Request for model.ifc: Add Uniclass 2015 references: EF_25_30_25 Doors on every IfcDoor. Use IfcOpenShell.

First a look at what the model holds.

```python
import ifcopenshell

model = ifcopenshell.open("model.ifc")
print(model.schema)
print("classifications:", [c.Name for c in model.by_type("IfcClassification")])
for ifc_class in ("IfcDoor", "IfcRoof", "IfcStair", "IfcWall", "IfcWindow"):
    print(ifc_class, len(model.by_type(ifc_class)))
```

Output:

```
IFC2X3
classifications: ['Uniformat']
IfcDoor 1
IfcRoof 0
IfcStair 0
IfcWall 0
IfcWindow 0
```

```python
import ifcopenshell
import ifcopenshell.api.classification

model = ifcopenshell.open("model.ifc")

# IFC2X3 requires Source and Edition and has no link from the project to the system.
system = model.create_entity("IfcClassification", Source="NBS", Edition="2015", Name="Uniclass 2015")

codes = {
    "IfcDoor": ("EF_25_30_25", "Doors"),
}
for ifc_class, (code, name) in codes.items():
    products = model.by_type(ifc_class)
    ifcopenshell.api.classification.add_reference(
        model, products=products, classification=system, identification=code, name=name
    )
    print(code, len(products))

model.write("model_updated.ifc")
```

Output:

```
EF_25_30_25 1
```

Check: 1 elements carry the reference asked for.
